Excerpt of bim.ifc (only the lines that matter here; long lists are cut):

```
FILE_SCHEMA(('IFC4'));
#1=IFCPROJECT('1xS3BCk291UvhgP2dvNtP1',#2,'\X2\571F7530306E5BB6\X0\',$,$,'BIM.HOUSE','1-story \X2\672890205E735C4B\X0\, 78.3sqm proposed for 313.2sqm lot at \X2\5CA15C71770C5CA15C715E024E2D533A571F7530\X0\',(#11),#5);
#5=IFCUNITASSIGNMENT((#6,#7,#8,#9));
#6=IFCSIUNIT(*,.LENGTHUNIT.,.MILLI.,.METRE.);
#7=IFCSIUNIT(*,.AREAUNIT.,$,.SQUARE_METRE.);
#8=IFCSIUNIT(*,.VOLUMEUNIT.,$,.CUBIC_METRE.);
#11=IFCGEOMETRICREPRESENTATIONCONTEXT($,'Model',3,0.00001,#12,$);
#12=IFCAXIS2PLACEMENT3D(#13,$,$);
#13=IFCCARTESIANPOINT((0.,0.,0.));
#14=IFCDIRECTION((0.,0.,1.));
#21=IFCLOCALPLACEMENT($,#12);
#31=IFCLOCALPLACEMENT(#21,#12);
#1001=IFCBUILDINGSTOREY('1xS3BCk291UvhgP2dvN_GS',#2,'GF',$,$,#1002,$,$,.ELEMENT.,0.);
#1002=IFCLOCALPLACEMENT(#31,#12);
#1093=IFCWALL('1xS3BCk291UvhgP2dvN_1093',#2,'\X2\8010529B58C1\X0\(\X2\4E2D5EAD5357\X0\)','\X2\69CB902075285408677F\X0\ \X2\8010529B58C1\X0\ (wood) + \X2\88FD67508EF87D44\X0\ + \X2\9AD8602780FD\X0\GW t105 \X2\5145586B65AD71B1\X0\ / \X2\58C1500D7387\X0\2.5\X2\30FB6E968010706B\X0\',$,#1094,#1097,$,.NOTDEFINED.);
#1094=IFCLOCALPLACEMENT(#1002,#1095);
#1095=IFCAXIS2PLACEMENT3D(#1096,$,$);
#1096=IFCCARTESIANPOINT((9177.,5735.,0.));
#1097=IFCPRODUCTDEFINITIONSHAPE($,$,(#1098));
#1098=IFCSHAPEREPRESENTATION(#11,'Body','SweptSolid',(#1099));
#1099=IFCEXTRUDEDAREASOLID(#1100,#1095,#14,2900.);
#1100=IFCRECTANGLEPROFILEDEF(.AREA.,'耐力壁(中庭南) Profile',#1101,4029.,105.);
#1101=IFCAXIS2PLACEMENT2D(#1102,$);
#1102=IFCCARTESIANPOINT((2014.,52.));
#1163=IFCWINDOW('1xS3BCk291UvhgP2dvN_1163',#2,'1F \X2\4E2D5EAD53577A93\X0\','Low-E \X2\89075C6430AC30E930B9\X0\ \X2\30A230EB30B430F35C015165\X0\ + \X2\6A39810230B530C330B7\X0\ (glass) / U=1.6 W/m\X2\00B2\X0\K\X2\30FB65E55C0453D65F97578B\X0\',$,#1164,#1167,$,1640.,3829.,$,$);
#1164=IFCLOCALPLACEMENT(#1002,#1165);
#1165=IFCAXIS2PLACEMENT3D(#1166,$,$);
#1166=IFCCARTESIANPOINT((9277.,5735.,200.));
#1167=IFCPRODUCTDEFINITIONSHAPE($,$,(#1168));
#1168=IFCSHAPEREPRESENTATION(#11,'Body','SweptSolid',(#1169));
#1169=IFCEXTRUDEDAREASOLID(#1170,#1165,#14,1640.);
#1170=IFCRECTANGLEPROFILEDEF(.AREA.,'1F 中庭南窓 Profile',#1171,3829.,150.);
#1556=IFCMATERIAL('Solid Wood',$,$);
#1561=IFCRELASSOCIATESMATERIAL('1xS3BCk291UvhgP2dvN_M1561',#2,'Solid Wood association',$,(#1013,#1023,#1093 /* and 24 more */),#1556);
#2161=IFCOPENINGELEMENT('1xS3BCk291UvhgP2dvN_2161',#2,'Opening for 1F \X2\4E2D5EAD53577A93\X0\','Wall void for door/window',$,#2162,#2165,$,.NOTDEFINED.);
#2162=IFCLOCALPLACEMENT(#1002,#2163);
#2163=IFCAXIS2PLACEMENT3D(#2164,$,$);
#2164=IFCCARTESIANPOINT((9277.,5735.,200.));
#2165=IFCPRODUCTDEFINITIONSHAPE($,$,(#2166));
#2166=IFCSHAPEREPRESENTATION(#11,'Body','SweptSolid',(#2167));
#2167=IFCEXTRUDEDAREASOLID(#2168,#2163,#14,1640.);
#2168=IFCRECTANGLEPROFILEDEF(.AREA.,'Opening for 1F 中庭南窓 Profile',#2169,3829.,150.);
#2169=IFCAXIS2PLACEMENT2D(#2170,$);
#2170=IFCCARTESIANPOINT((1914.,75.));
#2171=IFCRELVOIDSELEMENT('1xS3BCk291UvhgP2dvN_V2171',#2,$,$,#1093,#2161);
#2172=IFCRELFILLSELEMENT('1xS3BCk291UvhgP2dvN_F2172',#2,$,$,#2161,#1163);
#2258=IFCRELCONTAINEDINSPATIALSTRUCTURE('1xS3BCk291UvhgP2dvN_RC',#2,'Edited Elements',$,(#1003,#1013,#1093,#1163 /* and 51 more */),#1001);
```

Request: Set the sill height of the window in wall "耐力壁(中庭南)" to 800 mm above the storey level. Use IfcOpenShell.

```python
import numpy as np
import ifcopenshell
import ifcopenshell.api.geometry
import ifcopenshell.geom
import ifcopenshell.util.element
import ifcopenshell.util.placement
import ifcopenshell.util.shape
import ifcopenshell.util.unit

model = ifcopenshell.open("bim.ifc")
unit_scale = ifcopenshell.util.unit.calculate_unit_scale(model)

window = model.by_id(1163)
opening = window.FillsVoids[0].RelatingOpeningElement
storey = ifcopenshell.util.element.get_container(window, ifc_class="IfcBuildingStorey")
level = ifcopenshell.util.placement.get_local_placement(storey.ObjectPlacement)[2, 3]

# The opening's origin need not be at the sill, so measure its lowest point.
shape = ifcopenshell.geom.create_shape(ifcopenshell.geom.settings(), opening)
bottom = ifcopenshell.util.shape.get_shape_bottom_elevation(shape, shape.geometry) / unit_scale
dz = level + 800.0 - bottom

shift = np.array([0.0, 0.0, dz])
# The window is not placed relative to its opening, so move both.
for product in (opening, window):
    matrix = ifcopenshell.util.placement.get_local_placement(product.ObjectPlacement)
    matrix[:3, 3] += shift
    ifcopenshell.api.geometry.edit_object_placement(model, product=product, matrix=matrix, is_si=False)

print(f"moved by {dz * unit_scale:+.3f} m")

model.write("bim_edited.ifc")
```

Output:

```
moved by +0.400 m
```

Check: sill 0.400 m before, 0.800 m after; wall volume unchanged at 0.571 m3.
